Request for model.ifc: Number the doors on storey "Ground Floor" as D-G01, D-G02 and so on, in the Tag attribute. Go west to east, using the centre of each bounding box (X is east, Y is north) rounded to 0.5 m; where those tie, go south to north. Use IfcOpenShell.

First a look at what the model holds.

```python
import ifcopenshell
import ifcopenshell.util.element
import ifcopenshell.util.placement

model = ifcopenshell.open("model.ifc")
print(model.schema)
storey = next(s for s in model.by_type("IfcBuildingStorey") if s.Name == "Ground Floor")
doors = [e for e in ifcopenshell.util.element.get_decomposition(storey) if e.is_a("IfcDoor")]
for e in sorted(doors, key=lambda e: e.id()):
    origin = ifcopenshell.util.placement.get_local_placement(e.ObjectPlacement)[:3, 3]
    print(e.id(), e.Tag, e.Name, origin.round(2) + 0.0, sep=" | ")
```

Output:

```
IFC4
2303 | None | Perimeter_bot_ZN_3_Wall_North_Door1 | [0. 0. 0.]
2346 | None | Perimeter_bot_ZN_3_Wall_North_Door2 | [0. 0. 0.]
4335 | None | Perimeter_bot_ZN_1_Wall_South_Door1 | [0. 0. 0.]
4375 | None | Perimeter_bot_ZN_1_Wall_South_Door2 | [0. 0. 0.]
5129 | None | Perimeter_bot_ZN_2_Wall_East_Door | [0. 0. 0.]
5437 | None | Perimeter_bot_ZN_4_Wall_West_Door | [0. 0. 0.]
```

```python
import ifcopenshell
import ifcopenshell.geom
import ifcopenshell.util.element
import ifcopenshell.util.shape

model = ifcopenshell.open("model.ifc")
settings = ifcopenshell.geom.settings()
settings.set("use-world-coords", True)


def centre(element):
    shape = ifcopenshell.geom.create_shape(settings, element)
    return ifcopenshell.util.shape.get_bbox_centroid(shape.geometry)


storey = next(s for s in model.by_type("IfcBuildingStorey") if s.Name == "Ground Floor")
doors = [e for e in ifcopenshell.util.element.get_decomposition(storey) if e.is_a("IfcDoor")]

# Insertion points can sit at a corner or the storey origin, so sort by the geometry (in metres).
centres = {e: centre(e) for e in doors}
doors.sort(key=lambda e: (round(centres[e][0] / 0.5), centres[e][1]))

for i, e in enumerate(doors, start=1):
    number = f"D-G{i:02d}"
    e.Tag = number
    print(e.id(), number)

model.write("model_updated.ifc")
```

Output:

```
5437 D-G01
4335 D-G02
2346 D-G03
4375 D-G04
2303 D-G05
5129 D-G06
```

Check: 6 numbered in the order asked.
